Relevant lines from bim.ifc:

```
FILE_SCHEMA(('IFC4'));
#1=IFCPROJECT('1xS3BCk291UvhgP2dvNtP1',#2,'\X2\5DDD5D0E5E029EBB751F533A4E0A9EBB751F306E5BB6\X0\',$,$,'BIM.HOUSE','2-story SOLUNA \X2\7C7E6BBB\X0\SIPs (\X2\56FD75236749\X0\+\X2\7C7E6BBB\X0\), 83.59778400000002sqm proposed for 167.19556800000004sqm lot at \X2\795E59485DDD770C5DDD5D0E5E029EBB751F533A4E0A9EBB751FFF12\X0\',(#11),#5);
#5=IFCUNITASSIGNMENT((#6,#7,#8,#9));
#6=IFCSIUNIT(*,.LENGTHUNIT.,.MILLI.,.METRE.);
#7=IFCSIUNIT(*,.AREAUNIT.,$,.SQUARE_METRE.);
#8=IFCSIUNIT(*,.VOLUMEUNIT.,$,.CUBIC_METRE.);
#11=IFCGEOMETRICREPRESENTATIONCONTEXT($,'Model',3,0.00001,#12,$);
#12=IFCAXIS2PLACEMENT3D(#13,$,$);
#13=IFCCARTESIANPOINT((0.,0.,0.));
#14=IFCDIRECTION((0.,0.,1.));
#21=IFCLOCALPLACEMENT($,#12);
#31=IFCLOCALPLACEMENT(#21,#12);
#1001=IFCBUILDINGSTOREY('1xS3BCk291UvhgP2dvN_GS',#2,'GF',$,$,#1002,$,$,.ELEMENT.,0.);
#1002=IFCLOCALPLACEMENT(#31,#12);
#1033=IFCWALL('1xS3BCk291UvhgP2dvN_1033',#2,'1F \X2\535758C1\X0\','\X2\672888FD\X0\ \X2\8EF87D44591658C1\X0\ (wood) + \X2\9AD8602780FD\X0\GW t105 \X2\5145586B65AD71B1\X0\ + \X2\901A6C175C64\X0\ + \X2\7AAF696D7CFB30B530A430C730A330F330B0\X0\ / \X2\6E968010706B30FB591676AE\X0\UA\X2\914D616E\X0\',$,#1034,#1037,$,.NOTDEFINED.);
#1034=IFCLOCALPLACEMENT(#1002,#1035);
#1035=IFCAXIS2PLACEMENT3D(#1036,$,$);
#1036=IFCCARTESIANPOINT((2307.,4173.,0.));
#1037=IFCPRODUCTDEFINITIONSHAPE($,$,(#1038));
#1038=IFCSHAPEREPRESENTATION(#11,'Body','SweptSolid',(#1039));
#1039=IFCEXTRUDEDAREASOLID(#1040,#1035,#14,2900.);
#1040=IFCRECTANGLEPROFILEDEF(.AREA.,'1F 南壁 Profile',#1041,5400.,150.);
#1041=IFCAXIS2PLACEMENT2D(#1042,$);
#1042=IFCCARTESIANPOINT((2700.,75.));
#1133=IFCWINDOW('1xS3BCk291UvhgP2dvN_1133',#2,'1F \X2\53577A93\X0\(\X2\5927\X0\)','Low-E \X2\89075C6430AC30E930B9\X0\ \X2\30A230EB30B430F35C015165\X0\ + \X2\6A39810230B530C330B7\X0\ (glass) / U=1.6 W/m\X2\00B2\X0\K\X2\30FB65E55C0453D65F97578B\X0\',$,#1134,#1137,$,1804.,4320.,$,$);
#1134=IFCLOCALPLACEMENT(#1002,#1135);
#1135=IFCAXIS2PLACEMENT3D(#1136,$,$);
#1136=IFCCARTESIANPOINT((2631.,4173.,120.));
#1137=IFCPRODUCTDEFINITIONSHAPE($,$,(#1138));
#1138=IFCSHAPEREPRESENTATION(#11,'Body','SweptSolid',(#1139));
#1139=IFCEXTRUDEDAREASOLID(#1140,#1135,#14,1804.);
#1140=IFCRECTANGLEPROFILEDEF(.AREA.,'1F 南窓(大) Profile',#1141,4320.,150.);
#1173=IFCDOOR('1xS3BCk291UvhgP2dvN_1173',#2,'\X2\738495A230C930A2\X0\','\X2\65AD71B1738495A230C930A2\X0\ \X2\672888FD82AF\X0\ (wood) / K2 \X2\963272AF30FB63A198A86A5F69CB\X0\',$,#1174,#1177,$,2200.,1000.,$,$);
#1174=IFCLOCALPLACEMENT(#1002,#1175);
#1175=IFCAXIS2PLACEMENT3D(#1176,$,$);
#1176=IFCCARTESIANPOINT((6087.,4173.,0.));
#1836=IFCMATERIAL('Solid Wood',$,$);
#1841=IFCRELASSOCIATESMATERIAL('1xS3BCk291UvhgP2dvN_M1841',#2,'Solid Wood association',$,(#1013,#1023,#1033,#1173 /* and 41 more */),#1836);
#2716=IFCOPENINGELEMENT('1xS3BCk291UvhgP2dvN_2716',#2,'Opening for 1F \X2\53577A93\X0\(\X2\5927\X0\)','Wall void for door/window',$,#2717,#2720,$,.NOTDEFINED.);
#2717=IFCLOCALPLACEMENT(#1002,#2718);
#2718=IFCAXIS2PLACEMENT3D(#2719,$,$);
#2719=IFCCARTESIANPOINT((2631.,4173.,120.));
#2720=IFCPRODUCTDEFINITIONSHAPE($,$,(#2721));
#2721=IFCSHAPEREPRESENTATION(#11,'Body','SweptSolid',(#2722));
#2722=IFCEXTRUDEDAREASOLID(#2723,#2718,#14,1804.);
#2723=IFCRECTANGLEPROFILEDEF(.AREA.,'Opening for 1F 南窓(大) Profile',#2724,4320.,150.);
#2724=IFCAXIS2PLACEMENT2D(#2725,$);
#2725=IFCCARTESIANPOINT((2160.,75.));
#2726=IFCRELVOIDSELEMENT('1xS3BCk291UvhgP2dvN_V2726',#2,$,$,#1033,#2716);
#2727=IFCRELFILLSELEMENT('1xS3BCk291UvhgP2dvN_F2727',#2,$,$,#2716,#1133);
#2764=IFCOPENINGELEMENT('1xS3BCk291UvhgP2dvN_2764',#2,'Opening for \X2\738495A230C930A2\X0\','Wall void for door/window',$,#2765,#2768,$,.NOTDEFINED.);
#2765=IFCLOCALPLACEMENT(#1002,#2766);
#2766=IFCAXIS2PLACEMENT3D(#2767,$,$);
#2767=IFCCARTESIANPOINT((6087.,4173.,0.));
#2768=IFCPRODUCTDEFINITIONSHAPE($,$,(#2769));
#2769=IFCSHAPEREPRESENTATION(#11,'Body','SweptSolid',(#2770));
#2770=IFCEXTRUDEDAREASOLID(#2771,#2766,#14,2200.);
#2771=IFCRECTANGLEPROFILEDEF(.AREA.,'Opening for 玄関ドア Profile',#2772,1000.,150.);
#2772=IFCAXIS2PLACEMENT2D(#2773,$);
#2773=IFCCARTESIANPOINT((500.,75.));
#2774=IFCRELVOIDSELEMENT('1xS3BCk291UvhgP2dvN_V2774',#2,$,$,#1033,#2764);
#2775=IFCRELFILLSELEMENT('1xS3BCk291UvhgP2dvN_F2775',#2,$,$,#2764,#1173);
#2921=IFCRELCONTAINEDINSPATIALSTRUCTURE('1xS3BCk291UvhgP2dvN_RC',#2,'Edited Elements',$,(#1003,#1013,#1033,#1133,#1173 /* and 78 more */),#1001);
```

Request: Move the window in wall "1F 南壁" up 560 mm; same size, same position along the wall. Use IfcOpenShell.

```python
import numpy as np
import ifcopenshell
import ifcopenshell.api.geometry
import ifcopenshell.util.placement
import ifcopenshell.util.unit

model = ifcopenshell.open("bim.ifc")
unit_scale = ifcopenshell.util.unit.calculate_unit_scale(model)

window = model.by_id(1133)
opening = window.FillsVoids[0].RelatingOpeningElement
dz = 0.56 / unit_scale

shift = np.array([0.0, 0.0, dz])
# The window is not placed relative to its opening, so move both.
for product in (opening, window):
    matrix = ifcopenshell.util.placement.get_local_placement(product.ObjectPlacement)
    matrix[:3, 3] += shift
    ifcopenshell.api.geometry.edit_object_placement(model, product=product, matrix=matrix, is_si=False)

print(f"moved by {dz * unit_scale:+.3f} m")

model.write("bim_v2.ifc")
```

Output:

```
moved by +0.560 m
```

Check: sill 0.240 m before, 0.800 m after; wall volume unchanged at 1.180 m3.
